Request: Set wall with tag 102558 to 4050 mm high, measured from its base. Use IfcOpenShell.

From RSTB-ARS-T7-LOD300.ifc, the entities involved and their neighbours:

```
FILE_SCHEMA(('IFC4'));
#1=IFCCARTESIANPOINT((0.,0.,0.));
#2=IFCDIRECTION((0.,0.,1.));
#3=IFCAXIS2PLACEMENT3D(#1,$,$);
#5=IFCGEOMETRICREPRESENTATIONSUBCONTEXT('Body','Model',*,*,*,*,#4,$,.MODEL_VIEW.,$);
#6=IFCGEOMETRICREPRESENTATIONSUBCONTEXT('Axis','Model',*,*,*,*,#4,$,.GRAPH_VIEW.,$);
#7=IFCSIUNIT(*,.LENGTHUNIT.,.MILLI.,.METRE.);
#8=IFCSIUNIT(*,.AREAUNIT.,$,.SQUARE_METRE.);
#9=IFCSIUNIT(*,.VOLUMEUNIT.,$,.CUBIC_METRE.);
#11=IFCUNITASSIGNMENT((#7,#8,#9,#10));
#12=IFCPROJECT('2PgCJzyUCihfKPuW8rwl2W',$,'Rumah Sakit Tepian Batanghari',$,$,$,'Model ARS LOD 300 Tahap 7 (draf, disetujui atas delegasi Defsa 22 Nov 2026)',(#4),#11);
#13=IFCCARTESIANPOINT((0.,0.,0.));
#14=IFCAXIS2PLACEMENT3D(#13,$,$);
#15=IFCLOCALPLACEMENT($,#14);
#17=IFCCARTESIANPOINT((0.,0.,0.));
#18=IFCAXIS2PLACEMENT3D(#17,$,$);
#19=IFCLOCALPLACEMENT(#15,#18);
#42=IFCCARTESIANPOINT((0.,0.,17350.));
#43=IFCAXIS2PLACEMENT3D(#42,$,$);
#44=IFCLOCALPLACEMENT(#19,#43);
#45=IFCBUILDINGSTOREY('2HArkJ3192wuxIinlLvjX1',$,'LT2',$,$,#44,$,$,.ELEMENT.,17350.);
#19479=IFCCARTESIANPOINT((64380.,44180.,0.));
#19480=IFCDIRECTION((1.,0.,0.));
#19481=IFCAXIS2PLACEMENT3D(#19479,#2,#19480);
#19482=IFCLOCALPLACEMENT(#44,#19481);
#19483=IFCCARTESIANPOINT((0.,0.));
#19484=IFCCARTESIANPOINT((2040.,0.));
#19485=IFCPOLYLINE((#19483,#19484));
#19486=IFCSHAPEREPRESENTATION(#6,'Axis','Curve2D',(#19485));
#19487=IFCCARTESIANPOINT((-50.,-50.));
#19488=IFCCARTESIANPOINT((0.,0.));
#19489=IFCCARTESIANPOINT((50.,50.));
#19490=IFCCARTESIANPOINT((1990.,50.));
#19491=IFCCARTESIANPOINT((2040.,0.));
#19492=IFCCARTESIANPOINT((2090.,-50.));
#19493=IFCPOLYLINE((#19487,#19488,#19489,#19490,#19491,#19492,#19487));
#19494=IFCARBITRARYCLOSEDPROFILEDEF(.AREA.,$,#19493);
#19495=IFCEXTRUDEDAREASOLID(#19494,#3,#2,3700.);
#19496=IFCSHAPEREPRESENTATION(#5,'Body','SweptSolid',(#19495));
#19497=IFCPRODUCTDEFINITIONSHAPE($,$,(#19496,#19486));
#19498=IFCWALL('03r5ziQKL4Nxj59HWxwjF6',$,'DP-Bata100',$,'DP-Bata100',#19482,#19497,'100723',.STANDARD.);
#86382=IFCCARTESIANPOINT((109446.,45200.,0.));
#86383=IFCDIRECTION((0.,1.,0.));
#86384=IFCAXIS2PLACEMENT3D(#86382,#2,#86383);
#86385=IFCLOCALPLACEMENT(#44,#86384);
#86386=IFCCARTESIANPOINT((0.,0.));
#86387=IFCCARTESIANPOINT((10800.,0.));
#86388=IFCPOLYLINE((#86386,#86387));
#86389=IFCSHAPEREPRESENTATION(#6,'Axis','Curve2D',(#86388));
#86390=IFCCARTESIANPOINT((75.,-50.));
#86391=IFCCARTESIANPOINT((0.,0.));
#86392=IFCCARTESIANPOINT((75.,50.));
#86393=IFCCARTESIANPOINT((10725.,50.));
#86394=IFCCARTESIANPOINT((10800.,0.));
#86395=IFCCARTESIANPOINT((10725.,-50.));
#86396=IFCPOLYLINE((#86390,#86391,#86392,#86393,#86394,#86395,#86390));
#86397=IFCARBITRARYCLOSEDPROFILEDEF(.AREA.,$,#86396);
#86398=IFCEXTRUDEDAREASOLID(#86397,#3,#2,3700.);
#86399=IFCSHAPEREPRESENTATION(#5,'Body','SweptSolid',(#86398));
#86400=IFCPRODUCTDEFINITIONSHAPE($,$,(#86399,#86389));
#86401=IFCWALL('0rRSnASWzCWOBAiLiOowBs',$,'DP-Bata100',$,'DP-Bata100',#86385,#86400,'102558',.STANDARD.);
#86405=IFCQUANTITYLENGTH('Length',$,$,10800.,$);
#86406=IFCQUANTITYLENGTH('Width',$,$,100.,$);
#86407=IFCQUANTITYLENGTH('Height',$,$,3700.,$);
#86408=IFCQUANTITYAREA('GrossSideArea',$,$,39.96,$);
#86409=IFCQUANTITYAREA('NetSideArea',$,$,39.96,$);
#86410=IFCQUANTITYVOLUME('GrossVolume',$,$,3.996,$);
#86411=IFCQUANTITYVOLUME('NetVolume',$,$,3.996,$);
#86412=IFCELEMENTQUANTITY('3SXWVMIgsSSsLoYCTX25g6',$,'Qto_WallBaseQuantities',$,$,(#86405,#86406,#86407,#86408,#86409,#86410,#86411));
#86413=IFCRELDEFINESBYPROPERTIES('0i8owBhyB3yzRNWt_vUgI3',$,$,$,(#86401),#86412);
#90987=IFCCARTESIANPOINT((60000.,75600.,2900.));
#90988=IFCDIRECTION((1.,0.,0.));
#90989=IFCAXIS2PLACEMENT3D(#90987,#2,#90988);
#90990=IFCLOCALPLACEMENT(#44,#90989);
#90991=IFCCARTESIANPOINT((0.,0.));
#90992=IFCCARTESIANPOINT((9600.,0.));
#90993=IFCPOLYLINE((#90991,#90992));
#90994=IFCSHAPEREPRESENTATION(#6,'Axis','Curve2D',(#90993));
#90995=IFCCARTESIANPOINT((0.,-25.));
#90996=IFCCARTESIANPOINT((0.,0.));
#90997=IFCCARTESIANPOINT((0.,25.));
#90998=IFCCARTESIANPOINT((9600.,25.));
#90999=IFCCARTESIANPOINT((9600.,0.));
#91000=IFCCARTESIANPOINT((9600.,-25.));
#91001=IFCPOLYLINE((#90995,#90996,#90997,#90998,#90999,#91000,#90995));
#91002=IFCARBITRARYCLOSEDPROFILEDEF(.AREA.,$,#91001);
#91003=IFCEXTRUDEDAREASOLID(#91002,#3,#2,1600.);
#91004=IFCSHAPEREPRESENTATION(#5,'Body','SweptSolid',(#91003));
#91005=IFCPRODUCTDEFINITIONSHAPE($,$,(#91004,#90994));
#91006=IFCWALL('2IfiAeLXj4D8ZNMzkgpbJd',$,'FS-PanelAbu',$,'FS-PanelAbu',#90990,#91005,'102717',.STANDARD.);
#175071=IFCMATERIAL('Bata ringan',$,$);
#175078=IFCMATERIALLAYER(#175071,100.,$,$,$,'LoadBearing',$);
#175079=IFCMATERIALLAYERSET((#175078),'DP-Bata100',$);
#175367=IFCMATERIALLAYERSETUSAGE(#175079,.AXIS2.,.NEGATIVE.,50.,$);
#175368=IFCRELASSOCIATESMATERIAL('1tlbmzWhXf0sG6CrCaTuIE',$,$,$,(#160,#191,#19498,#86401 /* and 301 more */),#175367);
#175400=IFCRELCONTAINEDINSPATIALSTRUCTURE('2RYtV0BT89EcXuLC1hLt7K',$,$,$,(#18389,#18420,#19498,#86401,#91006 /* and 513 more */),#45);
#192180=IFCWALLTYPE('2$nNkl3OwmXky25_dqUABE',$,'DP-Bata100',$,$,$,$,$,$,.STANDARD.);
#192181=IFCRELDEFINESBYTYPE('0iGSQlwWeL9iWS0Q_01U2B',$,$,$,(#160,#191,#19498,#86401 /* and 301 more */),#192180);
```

```python
import ifcopenshell
import ifcopenshell.api.pset
import ifcopenshell.geom
import ifcopenshell.util.element
import ifcopenshell.util.representation
import ifcopenshell.util.shape
import ifcopenshell.util.unit

model = ifcopenshell.open("RSTB-ARS-T7-LOD300.ifc")
unit_scale = ifcopenshell.util.unit.calculate_unit_scale(model)
area_scale = ifcopenshell.util.unit.calculate_unit_scale(model, "AREAUNIT")
volume_scale = ifcopenshell.util.unit.calculate_unit_scale(model, "VOLUMEUNIT")
settings = ifcopenshell.geom.settings()


def volume(element):
    """Net volume in cubic metres, openings subtracted."""
    shape = ifcopenshell.geom.create_shape(settings, element)
    return ifcopenshell.util.shape.get_volume(shape.geometry)


wall = model.by_guid("0rRSnASWzCWOBAiLiOowBs")
before = volume(wall)

body = ifcopenshell.util.representation.get_representation(wall, "Model", "Body")
solid = body.Items[0]
old_height = solid.Depth
solid.Depth = 4050.0
after = volume(wall)
thickness = 0.1  # wall thickness in metres

# Update the stored height, areas and volumes.
qto = model.by_id(ifcopenshell.util.element.get_pset(wall, "Qto_WallBaseQuantities", should_inherit=False)["id"])
ifcopenshell.api.pset.edit_qto(model, qto=qto, properties={
    "Height": solid.Depth,
    "GrossSideArea": ifcopenshell.util.element.get_pset(wall, "Qto_WallBaseQuantities", "GrossSideArea") * solid.Depth / old_height,
    "NetSideArea": after / thickness / area_scale,
    "GrossVolume": ifcopenshell.util.element.get_pset(wall, "Qto_WallBaseQuantities", "GrossVolume") * solid.Depth / old_height,
    "NetVolume": after / volume_scale,
})

print(f"height {old_height:g} -> {solid.Depth:g}, volume {before:.3f} -> {after:.3f} m3")

model.write("RSTB-ARS-T7-LOD300_v2.ifc")
```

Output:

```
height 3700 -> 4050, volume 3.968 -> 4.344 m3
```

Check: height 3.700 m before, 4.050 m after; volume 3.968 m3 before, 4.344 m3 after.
